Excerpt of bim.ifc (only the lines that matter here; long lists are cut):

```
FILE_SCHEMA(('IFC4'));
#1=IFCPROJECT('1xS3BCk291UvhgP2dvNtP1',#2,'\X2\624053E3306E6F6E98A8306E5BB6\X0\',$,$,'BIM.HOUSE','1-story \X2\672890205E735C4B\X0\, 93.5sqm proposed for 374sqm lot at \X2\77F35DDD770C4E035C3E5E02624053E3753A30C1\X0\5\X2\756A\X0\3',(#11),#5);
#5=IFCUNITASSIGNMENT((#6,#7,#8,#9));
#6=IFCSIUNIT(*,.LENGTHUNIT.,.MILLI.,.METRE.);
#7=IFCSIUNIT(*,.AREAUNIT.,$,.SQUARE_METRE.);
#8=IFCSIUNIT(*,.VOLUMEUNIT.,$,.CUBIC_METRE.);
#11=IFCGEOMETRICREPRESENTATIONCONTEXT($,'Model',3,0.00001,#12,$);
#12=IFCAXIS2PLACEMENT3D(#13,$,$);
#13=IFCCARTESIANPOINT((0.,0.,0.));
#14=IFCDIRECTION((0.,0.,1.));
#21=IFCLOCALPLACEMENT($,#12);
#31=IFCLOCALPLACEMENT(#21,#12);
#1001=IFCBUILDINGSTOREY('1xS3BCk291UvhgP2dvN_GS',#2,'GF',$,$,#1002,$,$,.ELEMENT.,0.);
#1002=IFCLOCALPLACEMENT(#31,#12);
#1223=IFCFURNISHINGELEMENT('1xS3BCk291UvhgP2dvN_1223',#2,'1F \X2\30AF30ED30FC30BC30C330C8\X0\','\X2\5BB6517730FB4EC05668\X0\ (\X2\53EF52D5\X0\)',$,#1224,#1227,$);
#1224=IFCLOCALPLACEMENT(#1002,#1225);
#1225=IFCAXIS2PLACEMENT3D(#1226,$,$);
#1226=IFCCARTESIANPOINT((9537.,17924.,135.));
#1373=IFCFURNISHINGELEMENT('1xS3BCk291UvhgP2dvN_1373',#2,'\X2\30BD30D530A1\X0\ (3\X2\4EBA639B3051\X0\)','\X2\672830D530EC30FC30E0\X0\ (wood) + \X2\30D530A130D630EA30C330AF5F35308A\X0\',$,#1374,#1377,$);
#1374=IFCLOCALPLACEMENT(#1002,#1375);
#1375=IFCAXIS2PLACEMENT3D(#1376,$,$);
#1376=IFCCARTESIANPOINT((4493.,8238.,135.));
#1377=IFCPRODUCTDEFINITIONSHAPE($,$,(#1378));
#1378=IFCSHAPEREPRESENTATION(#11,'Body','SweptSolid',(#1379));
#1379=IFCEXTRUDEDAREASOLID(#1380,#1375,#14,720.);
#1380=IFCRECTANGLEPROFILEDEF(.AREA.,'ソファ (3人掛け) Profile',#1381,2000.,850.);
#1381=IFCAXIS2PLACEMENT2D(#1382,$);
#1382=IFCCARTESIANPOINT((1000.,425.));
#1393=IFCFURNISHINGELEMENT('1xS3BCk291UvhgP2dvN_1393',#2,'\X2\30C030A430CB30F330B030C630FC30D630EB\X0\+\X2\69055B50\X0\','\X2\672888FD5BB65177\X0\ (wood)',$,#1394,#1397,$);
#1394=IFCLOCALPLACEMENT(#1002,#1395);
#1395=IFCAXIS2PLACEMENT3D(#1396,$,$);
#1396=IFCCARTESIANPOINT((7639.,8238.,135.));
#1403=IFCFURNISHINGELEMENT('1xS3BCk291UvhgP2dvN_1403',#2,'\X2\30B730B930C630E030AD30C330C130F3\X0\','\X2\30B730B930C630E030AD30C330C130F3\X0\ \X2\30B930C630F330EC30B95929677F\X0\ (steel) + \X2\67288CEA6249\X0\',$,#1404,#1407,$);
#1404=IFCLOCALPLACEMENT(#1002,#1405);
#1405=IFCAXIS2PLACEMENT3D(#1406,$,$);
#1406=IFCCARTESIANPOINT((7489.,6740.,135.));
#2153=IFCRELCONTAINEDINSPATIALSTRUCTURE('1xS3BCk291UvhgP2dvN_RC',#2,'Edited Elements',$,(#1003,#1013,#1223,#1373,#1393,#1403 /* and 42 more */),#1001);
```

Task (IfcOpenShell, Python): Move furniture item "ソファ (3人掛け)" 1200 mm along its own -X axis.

```python
import ifcopenshell
import ifcopenshell.api.geometry
import ifcopenshell.util.placement
import ifcopenshell.util.unit

model = ifcopenshell.open("bim.ifc")
unit_scale = ifcopenshell.util.unit.calculate_unit_scale(model)

item = model.by_guid("1xS3BCk291UvhgP2dvN_1373")
matrix = ifcopenshell.util.placement.get_local_placement(item.ObjectPlacement)
matrix[:3, 3] -= matrix[:3, 0] * 1.2 / unit_scale
ifcopenshell.api.geometry.edit_object_placement(model, product=item, matrix=matrix, is_si=False)

print(ifcopenshell.util.placement.get_local_placement(item.ObjectPlacement).round(3) + 0.0)

model.write("bim-out.ifc")
```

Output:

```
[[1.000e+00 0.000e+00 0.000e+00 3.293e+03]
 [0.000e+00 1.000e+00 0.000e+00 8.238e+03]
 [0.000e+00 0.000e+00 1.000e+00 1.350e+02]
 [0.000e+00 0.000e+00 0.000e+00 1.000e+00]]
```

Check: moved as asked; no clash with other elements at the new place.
